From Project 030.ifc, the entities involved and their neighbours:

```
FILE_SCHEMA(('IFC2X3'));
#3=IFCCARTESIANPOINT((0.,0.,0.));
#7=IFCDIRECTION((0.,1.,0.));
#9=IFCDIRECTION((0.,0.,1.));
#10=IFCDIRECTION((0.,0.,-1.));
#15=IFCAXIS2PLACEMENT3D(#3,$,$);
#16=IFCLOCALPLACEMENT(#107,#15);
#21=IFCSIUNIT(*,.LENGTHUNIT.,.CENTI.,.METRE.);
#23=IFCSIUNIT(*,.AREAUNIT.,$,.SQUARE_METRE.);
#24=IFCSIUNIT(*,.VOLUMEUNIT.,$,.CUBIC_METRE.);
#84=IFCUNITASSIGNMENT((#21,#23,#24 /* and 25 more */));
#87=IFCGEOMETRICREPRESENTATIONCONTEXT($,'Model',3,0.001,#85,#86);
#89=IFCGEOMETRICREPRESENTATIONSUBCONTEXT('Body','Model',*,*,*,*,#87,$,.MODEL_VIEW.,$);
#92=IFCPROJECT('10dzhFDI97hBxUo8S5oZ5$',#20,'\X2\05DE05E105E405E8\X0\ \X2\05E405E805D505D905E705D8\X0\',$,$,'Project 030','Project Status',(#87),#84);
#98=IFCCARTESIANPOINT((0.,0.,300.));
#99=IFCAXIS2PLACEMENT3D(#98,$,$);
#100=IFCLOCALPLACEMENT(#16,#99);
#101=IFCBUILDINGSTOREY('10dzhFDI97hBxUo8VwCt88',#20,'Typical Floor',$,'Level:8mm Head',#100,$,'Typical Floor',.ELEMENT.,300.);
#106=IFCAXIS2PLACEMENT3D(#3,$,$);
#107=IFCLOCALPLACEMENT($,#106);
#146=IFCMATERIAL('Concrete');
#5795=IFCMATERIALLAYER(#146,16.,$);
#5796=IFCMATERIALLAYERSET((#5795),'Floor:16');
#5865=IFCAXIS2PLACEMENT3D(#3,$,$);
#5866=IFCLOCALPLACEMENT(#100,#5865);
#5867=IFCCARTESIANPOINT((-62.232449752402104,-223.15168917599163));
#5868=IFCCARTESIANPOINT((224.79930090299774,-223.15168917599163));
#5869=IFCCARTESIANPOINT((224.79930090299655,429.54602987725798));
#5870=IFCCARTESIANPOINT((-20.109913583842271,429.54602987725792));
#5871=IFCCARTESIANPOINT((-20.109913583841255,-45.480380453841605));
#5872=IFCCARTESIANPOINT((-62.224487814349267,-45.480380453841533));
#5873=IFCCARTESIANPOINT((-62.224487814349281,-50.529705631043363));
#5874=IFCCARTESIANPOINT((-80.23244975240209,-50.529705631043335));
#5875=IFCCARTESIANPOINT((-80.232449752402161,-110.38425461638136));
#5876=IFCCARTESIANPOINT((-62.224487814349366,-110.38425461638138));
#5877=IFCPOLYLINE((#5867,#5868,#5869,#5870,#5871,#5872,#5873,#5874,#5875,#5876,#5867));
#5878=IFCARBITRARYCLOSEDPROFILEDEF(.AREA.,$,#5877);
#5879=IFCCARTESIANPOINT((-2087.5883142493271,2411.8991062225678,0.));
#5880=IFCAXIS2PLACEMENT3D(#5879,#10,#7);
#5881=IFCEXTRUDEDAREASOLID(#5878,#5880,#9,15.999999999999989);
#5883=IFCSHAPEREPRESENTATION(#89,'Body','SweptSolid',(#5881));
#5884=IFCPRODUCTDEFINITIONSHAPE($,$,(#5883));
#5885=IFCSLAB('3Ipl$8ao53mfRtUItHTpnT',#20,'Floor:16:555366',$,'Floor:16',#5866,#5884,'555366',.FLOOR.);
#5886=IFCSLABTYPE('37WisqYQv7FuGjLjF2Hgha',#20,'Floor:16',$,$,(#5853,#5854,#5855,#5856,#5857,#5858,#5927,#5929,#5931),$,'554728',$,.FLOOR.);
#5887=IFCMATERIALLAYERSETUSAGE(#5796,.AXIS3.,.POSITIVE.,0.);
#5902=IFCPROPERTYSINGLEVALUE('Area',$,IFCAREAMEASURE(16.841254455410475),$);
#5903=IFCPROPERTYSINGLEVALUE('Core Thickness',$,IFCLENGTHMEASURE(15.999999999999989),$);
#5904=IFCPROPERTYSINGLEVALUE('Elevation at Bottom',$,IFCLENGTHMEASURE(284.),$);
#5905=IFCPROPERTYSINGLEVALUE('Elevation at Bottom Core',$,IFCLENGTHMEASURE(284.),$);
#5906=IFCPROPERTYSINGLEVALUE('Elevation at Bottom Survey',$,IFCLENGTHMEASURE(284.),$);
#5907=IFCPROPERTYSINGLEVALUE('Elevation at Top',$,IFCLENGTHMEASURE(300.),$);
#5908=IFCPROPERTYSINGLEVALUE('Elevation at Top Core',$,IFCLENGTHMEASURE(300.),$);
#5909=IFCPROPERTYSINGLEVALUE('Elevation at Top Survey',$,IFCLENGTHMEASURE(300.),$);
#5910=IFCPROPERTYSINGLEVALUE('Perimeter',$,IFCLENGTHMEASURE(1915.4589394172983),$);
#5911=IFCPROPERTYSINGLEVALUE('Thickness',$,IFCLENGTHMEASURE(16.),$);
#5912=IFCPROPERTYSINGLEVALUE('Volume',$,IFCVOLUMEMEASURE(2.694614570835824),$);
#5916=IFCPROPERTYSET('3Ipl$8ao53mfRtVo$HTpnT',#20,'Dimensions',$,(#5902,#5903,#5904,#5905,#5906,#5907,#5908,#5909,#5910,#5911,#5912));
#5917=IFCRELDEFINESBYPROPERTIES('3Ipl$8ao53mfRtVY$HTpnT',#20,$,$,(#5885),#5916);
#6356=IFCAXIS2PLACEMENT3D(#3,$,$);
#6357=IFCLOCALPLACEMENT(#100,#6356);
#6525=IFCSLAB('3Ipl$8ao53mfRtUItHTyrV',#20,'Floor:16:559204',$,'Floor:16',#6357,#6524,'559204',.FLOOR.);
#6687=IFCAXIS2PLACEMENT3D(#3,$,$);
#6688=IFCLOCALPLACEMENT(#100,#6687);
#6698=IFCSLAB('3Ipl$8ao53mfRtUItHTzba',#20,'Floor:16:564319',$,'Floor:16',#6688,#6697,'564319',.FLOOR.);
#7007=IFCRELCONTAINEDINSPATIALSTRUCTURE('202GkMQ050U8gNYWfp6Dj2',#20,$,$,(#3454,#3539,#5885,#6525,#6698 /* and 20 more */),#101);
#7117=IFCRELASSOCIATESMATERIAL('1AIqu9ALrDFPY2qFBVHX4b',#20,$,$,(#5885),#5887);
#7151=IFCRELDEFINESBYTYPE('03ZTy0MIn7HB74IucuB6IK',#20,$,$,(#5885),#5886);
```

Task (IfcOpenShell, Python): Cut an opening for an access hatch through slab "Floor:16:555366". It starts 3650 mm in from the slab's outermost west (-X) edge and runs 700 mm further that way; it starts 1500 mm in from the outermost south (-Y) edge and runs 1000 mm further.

```python
import numpy as np
import ifcopenshell
import ifcopenshell.api.feature
import ifcopenshell.api.geometry
import ifcopenshell.api.pset
import ifcopenshell.api.root
import ifcopenshell.geom
import ifcopenshell.util.element
import ifcopenshell.util.placement
import ifcopenshell.util.representation
import ifcopenshell.util.shape
import ifcopenshell.util.unit

model = ifcopenshell.open("Project 030.ifc")
unit_scale = ifcopenshell.util.unit.calculate_unit_scale(model)
area_scale = ifcopenshell.util.unit.calculate_unit_scale(model, "AREAUNIT")
volume_scale = ifcopenshell.util.unit.calculate_unit_scale(model, "VOLUMEUNIT")
settings = ifcopenshell.geom.settings()


def volume(element):
    """Net volume in cubic metres, openings subtracted."""
    shape = ifcopenshell.geom.create_shape(settings, element)
    return ifcopenshell.util.shape.get_volume(shape.geometry)


slab = model.by_id(5885)
before = volume(slab)

# Extent in the slab's own axes, in metres. The edges named are its -X and -Y sides.
slab_shape = ifcopenshell.geom.create_shape(settings, slab)
vertices = ifcopenshell.util.shape.get_vertices(slab_shape.geometry)
x_min, y_min, bottom = vertices.min(axis=0)
top = vertices[:, 2].max()

opening = ifcopenshell.api.root.create_entity(model, ifc_class="IfcOpeningElement", name="Access hatch opening")
context = ifcopenshell.util.representation.get_context(model, "Model", "Body", "MODEL_VIEW")
width, depth = 0.7, 1
outline = [(0.0, 0.0), (width, 0.0), (width, depth), (0.0, depth), (0.0, 0.0)]
# Overshoot both faces by 50 mm so the cut is clean.
shape = ifcopenshell.api.geometry.add_slab_representation(
    model, context=context, depth=top - bottom + 0.1, polyline=outline
)
ifcopenshell.api.geometry.assign_representation(model, product=opening, representation=shape)

matrix = ifcopenshell.util.placement.get_local_placement(slab.ObjectPlacement)
matrix[:, 3] = matrix @ np.append(np.array([x_min + 3.65, y_min + 1.5, bottom - 0.05]) / unit_scale, 1.0)
ifcopenshell.api.geometry.edit_object_placement(model, product=opening, matrix=matrix, is_si=False)
ifcopenshell.api.feature.add_feature(model, feature=opening, element=slab)

after = volume(slab)

# Update the slab's stored quantities.
pset = model.by_id(ifcopenshell.util.element.get_pset(slab, "Dimensions", should_inherit=False)["id"])
ifcopenshell.api.pset.edit_pset(model, pset=pset, properties={
    "Area": model.create_entity("IfcAreaMeasure", after / (top - bottom) / area_scale),
    "Volume": model.create_entity("IfcVolumeMeasure", after / volume_scale),
})

print(f"slab volume {before:.3f} -> {after:.3f} m3")

model.write("Project 030_v2.ifc")
```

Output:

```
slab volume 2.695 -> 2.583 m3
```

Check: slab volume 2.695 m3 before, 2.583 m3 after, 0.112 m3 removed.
